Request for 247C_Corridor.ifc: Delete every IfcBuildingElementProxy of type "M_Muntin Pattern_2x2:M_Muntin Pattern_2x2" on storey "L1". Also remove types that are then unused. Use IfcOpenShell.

First a look at what the model holds.

```python
import ifcopenshell
import ifcopenshell.util.element

model = ifcopenshell.open("247C_Corridor.ifc")
print(model.schema)
storey = next(s for s in model.by_type("IfcBuildingStorey") if s.Name == "L1")
proxies = [e for e in ifcopenshell.util.element.get_decomposition(storey) if e.is_a("IfcBuildingElementProxy")]
seen = {}
for e in proxies:
    element_type = ifcopenshell.util.element.get_type(e)
    name = element_type.Name if element_type not in (None, e) else None
    seen[name] = seen.get(name, 0) + 1
for name, count in sorted(seen.items(), key=str):
    print(count, "x", name)
```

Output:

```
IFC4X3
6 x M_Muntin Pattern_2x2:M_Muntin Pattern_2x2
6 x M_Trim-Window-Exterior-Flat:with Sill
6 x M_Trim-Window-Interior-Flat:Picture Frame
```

```python
import ifcopenshell
import ifcopenshell.api.root
import ifcopenshell.util.element

model = ifcopenshell.open("247C_Corridor.ifc")

storey = next(s for s in model.by_type("IfcBuildingStorey") if s.Name == "L1")
proxies = [e for e in ifcopenshell.util.element.get_decomposition(storey) if e.is_a("IfcBuildingElementProxy")]
targets = [e for e in proxies if (t := ifcopenshell.util.element.get_type(e)) not in (None, e) and t.Name == "M_Muntin Pattern_2x2:M_Muntin Pattern_2x2"]
types = {ifcopenshell.util.element.get_type(e) for e in targets} - {None, *targets}

for e in targets:
    ifcopenshell.api.root.remove_product(model, product=e)
print(len(targets), "removed")

unused = [t for t in types if not ifcopenshell.util.element.get_types(t)]
for t in unused:
    ifcopenshell.api.root.remove_product(model, product=t)
print(len(unused), "unused types removed")

model.write("247C_Corridor-out.ifc")
```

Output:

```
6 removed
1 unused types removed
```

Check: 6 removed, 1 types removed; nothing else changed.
